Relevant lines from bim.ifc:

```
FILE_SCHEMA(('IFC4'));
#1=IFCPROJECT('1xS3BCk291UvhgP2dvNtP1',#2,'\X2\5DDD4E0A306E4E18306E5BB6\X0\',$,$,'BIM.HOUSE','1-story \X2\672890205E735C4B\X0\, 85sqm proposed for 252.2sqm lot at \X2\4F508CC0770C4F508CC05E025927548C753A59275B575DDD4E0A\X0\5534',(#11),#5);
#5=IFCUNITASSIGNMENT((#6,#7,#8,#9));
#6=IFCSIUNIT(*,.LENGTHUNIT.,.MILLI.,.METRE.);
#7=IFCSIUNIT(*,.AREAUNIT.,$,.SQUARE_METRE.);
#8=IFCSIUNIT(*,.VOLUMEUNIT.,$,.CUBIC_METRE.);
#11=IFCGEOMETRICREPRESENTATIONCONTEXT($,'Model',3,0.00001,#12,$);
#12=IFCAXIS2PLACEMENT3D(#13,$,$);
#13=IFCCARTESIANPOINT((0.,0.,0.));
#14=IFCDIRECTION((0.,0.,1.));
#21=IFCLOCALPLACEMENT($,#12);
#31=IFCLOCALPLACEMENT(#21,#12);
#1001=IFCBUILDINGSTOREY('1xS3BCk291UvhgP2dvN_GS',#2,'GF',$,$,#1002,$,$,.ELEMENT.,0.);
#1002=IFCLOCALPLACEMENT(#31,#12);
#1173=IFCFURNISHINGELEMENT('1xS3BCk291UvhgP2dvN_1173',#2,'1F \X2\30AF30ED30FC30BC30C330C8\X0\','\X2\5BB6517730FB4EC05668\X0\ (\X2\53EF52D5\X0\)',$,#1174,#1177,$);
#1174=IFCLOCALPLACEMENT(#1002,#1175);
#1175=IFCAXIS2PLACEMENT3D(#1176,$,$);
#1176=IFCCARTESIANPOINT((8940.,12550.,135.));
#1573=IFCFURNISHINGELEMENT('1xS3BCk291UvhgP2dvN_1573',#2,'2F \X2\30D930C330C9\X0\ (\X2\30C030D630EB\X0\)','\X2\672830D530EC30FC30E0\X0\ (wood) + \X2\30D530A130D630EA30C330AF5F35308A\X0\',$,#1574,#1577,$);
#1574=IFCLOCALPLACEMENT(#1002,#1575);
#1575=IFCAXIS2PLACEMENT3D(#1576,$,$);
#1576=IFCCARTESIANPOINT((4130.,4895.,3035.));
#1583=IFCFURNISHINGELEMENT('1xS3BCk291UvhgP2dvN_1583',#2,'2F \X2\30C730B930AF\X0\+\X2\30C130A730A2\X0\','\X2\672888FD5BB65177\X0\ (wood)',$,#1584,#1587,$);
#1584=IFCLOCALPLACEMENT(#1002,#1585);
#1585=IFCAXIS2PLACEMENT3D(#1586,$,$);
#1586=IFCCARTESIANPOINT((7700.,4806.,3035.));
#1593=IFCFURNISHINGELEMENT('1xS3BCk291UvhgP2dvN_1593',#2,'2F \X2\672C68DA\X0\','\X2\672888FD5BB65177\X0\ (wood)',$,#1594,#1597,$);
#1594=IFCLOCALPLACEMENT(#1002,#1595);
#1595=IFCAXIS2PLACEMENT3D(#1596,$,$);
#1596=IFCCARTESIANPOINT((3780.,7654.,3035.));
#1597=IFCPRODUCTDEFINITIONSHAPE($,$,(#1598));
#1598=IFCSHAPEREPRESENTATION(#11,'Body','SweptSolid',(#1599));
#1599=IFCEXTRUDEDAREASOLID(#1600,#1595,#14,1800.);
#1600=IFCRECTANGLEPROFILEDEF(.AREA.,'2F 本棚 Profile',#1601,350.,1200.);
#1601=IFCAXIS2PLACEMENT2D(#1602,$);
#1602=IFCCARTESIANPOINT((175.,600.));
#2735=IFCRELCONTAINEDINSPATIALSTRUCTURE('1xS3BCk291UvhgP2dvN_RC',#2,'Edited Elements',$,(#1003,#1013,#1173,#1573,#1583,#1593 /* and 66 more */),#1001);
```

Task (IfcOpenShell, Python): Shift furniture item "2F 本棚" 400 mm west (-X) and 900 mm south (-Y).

```python
import ifcopenshell
import ifcopenshell.api.geometry
import ifcopenshell.util.placement

model = ifcopenshell.open("bim.ifc")

item = model.by_id(1593)
matrix = ifcopenshell.util.placement.get_local_placement(item.ObjectPlacement)
matrix[0, 3] -= 400.0
matrix[1, 3] -= 900.0
ifcopenshell.api.geometry.edit_object_placement(model, product=item, matrix=matrix, is_si=False)

print(ifcopenshell.util.placement.get_local_placement(item.ObjectPlacement).round(3) + 0.0)

model.write("bim_updated.ifc")
```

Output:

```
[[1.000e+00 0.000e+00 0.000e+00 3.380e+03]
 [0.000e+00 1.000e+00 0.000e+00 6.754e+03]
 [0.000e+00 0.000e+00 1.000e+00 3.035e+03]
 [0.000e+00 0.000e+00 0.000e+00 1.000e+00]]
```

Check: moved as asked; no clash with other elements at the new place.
